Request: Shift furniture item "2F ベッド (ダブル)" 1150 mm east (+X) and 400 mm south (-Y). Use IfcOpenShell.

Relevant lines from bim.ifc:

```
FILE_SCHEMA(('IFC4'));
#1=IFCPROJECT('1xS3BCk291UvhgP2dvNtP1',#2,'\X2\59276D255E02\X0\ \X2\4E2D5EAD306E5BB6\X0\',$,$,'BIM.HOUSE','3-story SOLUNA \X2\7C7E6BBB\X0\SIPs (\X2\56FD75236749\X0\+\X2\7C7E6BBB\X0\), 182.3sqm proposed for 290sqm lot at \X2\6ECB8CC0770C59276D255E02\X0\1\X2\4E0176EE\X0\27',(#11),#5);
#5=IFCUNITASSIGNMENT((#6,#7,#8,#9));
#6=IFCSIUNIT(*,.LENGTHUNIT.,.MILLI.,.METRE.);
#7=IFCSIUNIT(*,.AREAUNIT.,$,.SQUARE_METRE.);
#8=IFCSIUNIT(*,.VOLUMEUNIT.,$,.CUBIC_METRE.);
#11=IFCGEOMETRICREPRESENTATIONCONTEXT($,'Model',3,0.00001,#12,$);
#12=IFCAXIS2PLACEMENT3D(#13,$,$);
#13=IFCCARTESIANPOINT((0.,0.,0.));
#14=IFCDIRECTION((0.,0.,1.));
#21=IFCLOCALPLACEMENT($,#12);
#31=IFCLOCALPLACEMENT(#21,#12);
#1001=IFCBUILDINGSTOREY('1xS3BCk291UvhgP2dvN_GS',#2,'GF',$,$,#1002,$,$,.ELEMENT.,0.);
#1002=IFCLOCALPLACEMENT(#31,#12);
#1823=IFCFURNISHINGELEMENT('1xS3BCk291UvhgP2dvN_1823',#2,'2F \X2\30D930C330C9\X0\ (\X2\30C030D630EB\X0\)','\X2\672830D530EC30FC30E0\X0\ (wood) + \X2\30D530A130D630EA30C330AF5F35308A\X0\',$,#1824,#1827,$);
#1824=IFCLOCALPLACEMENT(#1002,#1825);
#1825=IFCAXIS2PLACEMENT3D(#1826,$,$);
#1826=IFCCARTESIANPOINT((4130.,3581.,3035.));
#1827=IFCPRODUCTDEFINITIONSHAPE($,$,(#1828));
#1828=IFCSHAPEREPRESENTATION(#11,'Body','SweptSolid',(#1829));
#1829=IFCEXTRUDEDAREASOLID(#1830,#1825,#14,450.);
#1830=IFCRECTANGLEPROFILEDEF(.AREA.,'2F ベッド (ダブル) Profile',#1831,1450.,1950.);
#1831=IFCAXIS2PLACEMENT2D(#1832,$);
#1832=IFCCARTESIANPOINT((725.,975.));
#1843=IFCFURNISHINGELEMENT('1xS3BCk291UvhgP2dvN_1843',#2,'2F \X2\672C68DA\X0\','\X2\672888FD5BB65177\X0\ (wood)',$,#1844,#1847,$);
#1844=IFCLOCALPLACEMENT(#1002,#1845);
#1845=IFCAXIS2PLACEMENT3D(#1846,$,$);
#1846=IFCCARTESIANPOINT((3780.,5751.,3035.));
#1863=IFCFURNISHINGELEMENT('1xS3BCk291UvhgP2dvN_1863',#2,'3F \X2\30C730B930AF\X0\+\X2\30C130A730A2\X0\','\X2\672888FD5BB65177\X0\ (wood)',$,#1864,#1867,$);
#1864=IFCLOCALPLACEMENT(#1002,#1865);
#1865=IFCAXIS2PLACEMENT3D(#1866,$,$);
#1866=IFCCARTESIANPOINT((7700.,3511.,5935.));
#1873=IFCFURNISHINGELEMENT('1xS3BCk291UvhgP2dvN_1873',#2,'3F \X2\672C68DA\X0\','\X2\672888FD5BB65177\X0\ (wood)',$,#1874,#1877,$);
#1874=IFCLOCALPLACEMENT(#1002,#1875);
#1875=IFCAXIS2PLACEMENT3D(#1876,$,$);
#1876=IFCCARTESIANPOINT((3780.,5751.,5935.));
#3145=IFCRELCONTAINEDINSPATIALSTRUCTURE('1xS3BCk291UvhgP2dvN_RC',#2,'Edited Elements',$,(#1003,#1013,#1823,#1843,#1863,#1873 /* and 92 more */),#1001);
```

```python
import ifcopenshell
import ifcopenshell.api.geometry
import ifcopenshell.util.placement
import ifcopenshell.util.unit

model = ifcopenshell.open("bim.ifc")
unit_scale = ifcopenshell.util.unit.calculate_unit_scale(model)

item = model.by_guid("1xS3BCk291UvhgP2dvN_1823")
matrix = ifcopenshell.util.placement.get_local_placement(item.ObjectPlacement)
matrix[0, 3] += 1.15 / unit_scale
matrix[1, 3] -= 0.4 / unit_scale
ifcopenshell.api.geometry.edit_object_placement(model, product=item, matrix=matrix, is_si=False)

print(ifcopenshell.util.placement.get_local_placement(item.ObjectPlacement).round(3) + 0.0)

model.write("bim_updated.ifc")
```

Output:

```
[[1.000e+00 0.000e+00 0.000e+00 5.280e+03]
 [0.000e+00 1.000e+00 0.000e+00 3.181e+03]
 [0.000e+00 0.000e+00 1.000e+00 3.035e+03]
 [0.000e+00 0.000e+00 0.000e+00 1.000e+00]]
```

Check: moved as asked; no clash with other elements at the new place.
